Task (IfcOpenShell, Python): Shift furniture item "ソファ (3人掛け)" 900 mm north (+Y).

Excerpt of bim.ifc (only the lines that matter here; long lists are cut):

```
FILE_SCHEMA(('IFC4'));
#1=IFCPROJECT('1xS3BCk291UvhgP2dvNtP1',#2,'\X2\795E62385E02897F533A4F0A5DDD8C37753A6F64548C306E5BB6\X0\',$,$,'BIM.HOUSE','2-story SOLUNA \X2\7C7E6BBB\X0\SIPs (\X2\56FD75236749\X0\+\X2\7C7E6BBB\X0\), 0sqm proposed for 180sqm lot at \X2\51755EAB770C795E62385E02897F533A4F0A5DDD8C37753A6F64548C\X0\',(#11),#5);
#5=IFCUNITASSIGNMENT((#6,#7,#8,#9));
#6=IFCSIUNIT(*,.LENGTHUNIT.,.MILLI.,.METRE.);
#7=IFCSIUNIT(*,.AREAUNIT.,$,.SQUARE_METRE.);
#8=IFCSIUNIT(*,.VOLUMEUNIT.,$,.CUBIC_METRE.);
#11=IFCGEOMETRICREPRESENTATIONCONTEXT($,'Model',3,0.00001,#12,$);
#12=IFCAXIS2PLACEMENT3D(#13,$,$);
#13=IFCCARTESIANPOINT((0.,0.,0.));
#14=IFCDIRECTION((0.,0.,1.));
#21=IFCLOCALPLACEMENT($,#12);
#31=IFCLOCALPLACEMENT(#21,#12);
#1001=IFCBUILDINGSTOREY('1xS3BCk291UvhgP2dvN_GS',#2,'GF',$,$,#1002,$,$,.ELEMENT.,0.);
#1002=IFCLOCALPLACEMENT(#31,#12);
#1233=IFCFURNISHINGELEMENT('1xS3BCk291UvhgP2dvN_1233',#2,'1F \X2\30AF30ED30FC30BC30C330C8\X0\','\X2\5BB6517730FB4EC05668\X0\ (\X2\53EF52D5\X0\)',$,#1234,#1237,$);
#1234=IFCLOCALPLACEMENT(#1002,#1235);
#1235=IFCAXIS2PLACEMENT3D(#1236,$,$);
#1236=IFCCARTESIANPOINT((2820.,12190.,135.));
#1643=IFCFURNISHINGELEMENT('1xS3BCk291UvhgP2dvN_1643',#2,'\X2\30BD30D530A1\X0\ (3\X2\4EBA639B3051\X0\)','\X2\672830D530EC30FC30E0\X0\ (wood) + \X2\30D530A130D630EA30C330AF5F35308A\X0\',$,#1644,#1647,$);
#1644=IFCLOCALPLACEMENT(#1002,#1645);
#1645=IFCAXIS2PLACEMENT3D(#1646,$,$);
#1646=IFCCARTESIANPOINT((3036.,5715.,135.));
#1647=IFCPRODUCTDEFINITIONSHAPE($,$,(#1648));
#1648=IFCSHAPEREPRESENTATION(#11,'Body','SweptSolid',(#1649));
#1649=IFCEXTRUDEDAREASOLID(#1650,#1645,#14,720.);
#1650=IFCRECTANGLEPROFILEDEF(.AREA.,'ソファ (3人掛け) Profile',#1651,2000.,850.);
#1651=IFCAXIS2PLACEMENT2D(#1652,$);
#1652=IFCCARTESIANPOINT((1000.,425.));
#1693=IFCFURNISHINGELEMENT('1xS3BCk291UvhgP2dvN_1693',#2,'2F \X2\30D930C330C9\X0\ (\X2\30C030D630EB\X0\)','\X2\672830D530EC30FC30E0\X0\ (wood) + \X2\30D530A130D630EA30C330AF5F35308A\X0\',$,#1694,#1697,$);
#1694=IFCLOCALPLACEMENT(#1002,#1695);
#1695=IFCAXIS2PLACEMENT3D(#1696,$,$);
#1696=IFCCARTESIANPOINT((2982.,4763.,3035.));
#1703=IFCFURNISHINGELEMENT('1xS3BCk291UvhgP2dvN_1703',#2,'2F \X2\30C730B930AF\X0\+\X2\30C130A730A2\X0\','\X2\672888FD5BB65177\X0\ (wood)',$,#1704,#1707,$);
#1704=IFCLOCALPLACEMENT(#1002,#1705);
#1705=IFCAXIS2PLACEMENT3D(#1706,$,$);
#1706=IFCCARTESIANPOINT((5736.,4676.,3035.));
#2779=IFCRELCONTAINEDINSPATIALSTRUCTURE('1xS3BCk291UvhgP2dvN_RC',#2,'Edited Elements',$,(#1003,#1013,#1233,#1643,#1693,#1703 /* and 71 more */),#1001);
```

```python
import ifcopenshell
import ifcopenshell.api.geometry
import ifcopenshell.util.placement
import ifcopenshell.util.unit

model = ifcopenshell.open("bim.ifc")
unit_scale = ifcopenshell.util.unit.calculate_unit_scale(model)

item = model.by_guid("1xS3BCk291UvhgP2dvN_1643")
matrix = ifcopenshell.util.placement.get_local_placement(item.ObjectPlacement)
matrix[1, 3] += 0.9 / unit_scale
ifcopenshell.api.geometry.edit_object_placement(model, product=item, matrix=matrix, is_si=False)

print(ifcopenshell.util.placement.get_local_placement(item.ObjectPlacement).round(3) + 0.0)

model.write("bim_updated.ifc")
```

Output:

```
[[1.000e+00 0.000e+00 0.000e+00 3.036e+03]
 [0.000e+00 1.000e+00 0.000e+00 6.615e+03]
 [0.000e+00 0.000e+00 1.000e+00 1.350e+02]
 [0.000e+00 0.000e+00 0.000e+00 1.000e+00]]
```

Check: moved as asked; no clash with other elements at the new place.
